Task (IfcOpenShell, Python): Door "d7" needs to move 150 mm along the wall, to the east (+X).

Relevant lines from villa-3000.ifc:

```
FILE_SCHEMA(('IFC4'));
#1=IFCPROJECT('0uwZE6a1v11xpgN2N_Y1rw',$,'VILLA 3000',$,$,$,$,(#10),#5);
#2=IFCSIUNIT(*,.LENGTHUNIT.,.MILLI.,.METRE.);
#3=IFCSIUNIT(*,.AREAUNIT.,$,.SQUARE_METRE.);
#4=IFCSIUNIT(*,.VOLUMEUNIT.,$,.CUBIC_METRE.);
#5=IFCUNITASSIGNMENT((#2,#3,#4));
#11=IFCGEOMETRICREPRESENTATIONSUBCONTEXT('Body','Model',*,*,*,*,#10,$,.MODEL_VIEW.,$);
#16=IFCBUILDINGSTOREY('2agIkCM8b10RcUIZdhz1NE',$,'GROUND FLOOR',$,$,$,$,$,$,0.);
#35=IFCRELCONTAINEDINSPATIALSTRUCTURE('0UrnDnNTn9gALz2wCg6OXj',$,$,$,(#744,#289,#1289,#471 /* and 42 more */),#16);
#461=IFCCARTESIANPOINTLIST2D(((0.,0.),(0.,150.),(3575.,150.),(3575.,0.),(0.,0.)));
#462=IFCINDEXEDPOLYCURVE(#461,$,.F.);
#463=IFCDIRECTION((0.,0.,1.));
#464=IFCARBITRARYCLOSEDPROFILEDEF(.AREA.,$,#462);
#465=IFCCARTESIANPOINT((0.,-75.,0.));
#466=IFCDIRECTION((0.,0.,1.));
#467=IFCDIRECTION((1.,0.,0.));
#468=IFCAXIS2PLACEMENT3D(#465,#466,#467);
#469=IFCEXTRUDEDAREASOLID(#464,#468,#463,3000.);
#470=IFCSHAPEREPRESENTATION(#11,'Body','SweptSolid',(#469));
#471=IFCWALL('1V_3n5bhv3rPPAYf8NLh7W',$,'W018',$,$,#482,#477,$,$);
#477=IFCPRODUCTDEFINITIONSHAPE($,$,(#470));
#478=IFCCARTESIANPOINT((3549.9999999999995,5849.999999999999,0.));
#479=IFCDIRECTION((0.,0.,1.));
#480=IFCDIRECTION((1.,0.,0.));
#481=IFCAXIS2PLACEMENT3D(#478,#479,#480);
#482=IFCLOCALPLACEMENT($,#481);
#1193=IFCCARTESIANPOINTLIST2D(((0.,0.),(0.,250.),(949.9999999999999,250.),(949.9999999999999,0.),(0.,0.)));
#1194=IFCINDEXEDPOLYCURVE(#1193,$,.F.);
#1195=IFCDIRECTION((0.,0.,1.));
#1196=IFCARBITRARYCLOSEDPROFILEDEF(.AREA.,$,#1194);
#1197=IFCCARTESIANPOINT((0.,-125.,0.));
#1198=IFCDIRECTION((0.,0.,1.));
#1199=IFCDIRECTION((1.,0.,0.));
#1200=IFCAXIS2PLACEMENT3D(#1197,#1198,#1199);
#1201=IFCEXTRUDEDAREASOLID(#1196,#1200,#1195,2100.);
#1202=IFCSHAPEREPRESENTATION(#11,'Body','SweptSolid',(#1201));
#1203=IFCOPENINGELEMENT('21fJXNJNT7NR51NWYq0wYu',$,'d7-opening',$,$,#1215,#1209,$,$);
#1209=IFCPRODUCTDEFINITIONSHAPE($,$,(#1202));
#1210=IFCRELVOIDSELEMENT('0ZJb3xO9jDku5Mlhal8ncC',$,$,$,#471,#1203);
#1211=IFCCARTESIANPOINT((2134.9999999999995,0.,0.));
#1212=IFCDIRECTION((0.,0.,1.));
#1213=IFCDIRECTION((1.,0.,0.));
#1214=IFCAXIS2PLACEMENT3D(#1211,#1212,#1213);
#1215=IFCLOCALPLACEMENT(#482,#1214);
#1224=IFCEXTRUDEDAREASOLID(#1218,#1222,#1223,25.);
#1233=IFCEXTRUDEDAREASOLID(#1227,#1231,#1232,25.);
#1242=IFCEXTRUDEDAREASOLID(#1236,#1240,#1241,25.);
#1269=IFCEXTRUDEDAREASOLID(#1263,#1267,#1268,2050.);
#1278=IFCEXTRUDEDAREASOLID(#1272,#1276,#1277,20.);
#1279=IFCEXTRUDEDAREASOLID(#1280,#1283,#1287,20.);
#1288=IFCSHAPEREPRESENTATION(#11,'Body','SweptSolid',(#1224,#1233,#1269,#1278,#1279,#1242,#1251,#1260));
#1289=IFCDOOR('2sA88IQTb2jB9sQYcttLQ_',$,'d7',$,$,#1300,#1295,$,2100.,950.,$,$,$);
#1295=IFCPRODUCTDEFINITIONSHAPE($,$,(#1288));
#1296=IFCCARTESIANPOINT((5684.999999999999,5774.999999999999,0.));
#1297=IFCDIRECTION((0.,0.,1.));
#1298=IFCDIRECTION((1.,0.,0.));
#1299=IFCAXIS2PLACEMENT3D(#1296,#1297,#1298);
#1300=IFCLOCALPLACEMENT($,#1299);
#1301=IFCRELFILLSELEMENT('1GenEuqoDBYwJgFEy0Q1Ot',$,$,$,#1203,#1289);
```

```python
import ifcopenshell
import ifcopenshell.api.geometry
import ifcopenshell.util.placement

model = ifcopenshell.open("villa-3000.ifc")

door = model.by_guid("2sA88IQTb2jB9sQYcttLQ_")
opening = door.FillsVoids[0].RelatingOpeningElement
wall = opening.VoidsElements[0].RelatingBuildingElement

wall_matrix = ifcopenshell.util.placement.get_local_placement(wall.ObjectPlacement)
shift = wall_matrix[:3, 0] * 150.0
before = ifcopenshell.util.placement.get_local_placement(door.ObjectPlacement)[:3, 3].copy()

# The door is not placed relative to its opening, so move both.
for product in (opening, door):
    matrix = ifcopenshell.util.placement.get_local_placement(product.ObjectPlacement)
    matrix[:3, 3] += shift
    ifcopenshell.api.geometry.edit_object_placement(model, product=product, matrix=matrix, is_si=False)

after = ifcopenshell.util.placement.get_local_placement(door.ObjectPlacement)[:3, 3]
print("door moved by", (after - before).round(3) + 0.0)

model.write("villa-3000_edited.ifc")
```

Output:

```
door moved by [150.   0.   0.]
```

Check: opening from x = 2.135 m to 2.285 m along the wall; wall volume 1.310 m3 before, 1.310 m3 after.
